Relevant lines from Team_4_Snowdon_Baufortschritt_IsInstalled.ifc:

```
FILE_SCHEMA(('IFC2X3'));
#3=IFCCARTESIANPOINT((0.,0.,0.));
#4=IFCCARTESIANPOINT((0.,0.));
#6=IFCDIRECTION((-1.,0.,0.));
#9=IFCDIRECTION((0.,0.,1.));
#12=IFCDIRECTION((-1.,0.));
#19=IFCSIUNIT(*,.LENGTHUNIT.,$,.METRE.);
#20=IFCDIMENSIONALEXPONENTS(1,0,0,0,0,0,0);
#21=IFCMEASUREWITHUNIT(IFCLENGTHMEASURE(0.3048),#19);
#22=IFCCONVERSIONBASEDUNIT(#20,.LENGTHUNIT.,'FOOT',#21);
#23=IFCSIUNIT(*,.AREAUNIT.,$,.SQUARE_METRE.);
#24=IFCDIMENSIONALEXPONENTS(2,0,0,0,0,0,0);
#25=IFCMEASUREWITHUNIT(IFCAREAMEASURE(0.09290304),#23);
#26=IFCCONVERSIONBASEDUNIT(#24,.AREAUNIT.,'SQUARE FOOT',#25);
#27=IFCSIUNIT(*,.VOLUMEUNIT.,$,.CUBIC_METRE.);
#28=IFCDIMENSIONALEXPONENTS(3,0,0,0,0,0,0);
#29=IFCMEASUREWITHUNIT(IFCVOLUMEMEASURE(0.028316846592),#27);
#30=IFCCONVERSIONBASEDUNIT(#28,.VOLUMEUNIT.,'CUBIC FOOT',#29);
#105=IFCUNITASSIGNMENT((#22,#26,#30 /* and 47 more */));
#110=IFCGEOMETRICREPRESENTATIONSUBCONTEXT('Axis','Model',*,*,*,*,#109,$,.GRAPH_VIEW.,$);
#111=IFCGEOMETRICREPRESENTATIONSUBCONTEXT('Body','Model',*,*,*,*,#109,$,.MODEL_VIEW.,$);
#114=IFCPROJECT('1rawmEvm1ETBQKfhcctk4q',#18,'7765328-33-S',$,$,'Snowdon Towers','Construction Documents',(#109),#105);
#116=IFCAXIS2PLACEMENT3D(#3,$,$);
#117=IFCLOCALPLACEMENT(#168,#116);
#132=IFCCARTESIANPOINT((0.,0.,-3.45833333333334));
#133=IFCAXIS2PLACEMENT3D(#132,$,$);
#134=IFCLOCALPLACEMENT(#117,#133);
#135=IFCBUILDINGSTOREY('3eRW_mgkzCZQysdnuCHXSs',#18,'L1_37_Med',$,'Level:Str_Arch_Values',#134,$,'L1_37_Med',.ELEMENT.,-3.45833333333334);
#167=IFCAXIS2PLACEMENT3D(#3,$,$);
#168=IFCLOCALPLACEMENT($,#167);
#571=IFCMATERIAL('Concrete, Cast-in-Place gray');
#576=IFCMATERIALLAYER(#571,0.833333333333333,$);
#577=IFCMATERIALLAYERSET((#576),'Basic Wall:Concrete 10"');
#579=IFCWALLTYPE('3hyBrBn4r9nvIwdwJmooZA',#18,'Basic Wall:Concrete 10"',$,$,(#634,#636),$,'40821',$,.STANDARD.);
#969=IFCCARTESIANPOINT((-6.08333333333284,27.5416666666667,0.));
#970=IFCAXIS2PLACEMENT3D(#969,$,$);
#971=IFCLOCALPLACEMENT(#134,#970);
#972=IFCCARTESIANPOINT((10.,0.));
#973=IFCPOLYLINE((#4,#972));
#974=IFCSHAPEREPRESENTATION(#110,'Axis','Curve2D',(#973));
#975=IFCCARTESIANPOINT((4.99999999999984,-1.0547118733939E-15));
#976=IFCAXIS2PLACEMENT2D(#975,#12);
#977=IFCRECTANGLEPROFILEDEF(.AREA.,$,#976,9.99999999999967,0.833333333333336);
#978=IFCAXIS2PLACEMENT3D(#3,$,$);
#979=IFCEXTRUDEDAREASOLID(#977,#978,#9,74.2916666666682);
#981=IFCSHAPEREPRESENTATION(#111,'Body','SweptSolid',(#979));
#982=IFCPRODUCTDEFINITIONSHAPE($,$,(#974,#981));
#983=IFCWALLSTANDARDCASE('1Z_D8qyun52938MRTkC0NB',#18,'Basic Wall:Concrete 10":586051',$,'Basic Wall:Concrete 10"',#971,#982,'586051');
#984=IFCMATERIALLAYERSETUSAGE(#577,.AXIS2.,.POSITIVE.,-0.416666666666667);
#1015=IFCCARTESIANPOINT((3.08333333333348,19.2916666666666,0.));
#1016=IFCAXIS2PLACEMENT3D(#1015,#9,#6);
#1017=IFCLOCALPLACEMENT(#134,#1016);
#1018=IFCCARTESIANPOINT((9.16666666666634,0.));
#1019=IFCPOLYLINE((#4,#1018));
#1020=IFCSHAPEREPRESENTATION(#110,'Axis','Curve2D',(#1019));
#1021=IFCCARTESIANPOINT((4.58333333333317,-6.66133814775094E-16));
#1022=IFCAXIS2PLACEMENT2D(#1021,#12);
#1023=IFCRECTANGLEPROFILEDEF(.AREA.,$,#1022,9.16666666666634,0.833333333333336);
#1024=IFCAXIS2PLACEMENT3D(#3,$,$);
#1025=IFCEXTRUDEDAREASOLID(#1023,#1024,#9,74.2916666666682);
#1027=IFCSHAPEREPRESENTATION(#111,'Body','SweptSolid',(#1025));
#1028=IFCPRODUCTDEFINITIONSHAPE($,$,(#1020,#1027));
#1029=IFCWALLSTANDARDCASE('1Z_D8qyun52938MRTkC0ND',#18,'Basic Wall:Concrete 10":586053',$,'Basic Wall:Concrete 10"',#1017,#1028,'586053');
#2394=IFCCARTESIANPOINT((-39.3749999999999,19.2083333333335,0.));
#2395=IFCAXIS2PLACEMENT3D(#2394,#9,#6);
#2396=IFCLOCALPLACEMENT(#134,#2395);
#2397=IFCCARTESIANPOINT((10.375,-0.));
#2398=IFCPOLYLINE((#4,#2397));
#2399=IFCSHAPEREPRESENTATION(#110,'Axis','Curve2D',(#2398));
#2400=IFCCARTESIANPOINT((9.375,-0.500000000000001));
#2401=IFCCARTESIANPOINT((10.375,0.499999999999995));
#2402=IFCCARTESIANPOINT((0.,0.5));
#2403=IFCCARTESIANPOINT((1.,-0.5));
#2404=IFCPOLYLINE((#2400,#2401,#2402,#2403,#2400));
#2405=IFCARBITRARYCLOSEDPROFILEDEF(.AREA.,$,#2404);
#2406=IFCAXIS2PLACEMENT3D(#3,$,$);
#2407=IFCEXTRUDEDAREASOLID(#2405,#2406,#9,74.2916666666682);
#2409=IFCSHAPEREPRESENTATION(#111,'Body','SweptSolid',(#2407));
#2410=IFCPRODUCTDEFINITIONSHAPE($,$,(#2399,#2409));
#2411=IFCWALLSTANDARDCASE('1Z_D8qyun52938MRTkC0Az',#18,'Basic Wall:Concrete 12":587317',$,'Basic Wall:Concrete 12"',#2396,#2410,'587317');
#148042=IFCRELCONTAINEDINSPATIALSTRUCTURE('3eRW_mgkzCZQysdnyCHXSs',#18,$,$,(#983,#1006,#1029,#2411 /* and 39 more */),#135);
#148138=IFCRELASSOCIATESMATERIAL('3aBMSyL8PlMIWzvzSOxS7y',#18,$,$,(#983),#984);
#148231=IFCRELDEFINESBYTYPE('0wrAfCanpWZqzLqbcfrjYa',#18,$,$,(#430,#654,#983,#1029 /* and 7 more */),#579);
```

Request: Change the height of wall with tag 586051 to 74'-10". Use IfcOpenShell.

```python
import ifcopenshell
import ifcopenshell.geom
import ifcopenshell.util.representation
import ifcopenshell.util.shape
import ifcopenshell.util.unit

model = ifcopenshell.open("Team_4_Snowdon_Baufortschritt_IsInstalled.ifc")
unit_scale = ifcopenshell.util.unit.calculate_unit_scale(model)
settings = ifcopenshell.geom.settings()


def volume(element):
    """Net volume in cubic metres, openings subtracted."""
    shape = ifcopenshell.geom.create_shape(settings, element)
    return ifcopenshell.util.shape.get_volume(shape.geometry)


wall = model.by_guid("1Z_D8qyun52938MRTkC0NB")
before = volume(wall)

body = ifcopenshell.util.representation.get_representation(wall, "Model", "Body")
solid = body.Items[0]
old_height = solid.Depth
solid.Depth = 898 * 0.0254 / unit_scale
after = volume(wall)

print(f"height {old_height:g} -> {solid.Depth:g}, volume {before:.3f} -> {after:.3f} m3")

model.write("Team_4_Snowdon_Baufortschritt_IsInstalled-out.ifc")
```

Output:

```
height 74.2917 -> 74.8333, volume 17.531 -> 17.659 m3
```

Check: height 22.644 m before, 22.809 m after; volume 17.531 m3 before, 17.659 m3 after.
